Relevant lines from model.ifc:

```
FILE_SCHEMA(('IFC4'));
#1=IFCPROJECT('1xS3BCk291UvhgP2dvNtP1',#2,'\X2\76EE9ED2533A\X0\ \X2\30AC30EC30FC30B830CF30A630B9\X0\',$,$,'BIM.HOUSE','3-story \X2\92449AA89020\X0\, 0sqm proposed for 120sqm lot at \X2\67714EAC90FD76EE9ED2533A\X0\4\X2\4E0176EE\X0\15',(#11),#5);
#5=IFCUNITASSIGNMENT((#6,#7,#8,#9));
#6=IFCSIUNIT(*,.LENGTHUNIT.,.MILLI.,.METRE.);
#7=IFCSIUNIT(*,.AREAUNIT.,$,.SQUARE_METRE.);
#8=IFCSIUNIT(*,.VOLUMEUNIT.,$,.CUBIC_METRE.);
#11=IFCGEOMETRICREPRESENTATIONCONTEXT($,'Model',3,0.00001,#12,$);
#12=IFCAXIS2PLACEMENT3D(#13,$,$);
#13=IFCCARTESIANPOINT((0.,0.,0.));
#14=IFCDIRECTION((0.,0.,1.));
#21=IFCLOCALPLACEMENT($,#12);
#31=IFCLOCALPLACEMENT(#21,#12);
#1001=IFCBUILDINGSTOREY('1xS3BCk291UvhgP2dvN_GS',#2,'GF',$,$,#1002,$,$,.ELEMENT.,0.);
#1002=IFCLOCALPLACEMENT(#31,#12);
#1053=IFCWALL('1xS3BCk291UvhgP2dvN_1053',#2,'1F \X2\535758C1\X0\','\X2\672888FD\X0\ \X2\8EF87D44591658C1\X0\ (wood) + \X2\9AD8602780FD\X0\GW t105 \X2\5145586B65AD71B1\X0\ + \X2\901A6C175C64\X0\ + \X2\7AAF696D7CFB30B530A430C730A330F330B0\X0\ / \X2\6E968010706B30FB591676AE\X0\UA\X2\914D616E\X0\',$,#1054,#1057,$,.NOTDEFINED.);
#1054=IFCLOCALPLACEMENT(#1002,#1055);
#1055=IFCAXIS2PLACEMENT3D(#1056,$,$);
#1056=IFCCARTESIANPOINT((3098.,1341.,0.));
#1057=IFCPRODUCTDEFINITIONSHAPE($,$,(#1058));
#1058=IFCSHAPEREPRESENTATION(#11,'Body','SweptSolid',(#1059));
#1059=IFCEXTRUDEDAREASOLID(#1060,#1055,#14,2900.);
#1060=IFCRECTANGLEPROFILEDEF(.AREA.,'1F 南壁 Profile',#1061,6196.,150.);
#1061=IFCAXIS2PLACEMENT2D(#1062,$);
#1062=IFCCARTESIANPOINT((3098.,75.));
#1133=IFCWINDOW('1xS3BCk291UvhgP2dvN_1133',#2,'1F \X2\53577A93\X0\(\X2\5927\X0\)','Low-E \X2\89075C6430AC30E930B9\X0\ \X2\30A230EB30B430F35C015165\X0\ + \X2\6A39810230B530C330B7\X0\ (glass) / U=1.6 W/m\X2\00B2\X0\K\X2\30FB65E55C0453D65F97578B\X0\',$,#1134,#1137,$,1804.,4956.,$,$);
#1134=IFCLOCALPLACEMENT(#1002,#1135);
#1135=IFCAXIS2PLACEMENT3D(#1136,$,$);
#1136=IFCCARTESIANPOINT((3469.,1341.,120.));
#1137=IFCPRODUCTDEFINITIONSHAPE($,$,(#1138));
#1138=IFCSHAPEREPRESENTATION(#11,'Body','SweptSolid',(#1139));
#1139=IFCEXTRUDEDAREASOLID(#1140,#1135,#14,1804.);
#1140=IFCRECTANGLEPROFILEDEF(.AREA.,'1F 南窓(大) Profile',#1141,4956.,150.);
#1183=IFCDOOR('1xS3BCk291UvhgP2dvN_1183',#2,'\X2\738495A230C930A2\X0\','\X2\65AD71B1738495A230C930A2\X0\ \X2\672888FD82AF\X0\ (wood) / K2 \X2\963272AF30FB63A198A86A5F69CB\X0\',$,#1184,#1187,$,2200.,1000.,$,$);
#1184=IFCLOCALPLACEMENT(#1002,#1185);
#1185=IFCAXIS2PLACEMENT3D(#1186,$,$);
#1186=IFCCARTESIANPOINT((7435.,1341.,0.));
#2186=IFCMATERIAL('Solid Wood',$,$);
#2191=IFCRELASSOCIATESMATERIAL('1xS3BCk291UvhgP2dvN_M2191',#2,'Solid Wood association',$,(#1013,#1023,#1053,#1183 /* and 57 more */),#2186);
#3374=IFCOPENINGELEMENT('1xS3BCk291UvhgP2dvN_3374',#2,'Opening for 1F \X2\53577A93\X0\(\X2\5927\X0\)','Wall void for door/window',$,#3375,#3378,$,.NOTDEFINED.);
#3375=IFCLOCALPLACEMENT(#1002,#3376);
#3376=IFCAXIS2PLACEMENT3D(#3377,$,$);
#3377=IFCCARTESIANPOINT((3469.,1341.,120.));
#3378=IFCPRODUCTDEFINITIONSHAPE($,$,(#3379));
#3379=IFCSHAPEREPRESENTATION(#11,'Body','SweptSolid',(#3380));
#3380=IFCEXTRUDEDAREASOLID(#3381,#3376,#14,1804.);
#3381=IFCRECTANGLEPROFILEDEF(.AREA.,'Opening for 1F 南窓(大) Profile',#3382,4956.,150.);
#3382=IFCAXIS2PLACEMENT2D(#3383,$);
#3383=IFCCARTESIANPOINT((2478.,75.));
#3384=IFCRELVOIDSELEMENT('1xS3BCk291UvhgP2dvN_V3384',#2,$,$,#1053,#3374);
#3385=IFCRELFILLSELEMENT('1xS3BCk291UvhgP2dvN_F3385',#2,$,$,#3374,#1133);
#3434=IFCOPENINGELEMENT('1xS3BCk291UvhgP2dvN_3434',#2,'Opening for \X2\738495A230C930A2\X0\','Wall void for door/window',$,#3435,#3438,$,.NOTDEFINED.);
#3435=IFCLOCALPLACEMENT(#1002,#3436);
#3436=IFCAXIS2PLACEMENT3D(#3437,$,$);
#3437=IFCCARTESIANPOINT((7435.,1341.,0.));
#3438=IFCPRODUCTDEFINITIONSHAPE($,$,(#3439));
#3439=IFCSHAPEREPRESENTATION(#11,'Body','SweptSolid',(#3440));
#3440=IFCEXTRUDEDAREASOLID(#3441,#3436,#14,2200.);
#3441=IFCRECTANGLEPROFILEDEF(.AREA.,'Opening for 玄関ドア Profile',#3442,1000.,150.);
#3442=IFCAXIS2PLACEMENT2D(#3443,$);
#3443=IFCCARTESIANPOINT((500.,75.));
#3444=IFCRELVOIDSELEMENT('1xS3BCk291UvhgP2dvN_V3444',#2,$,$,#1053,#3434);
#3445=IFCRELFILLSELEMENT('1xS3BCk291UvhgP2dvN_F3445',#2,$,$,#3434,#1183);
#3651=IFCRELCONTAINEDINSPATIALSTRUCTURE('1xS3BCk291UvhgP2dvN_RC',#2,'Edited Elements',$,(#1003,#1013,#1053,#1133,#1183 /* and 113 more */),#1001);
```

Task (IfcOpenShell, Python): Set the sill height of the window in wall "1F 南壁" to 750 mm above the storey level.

```python
import numpy as np
import ifcopenshell
import ifcopenshell.api.geometry
import ifcopenshell.geom
import ifcopenshell.util.element
import ifcopenshell.util.placement
import ifcopenshell.util.shape
import ifcopenshell.util.unit

model = ifcopenshell.open("model.ifc")
unit_scale = ifcopenshell.util.unit.calculate_unit_scale(model)

window = model.by_id(1133)
opening = window.FillsVoids[0].RelatingOpeningElement
storey = ifcopenshell.util.element.get_container(window, ifc_class="IfcBuildingStorey")
level = ifcopenshell.util.placement.get_local_placement(storey.ObjectPlacement)[2, 3]

# The opening's origin need not be at the sill, so measure its lowest point.
shape = ifcopenshell.geom.create_shape(ifcopenshell.geom.settings(), opening)
bottom = ifcopenshell.util.shape.get_shape_bottom_elevation(shape, shape.geometry) / unit_scale
dz = level + 0.75 / unit_scale - bottom

shift = np.array([0.0, 0.0, dz])
# The window is not placed relative to its opening, so move both.
for product in (opening, window):
    matrix = ifcopenshell.util.placement.get_local_placement(product.ObjectPlacement)
    matrix[:3, 3] += shift
    ifcopenshell.api.geometry.edit_object_placement(model, product=product, matrix=matrix, is_si=False)

print(f"moved by {dz * unit_scale:+.3f} m")

model.write("model-out.ifc")
```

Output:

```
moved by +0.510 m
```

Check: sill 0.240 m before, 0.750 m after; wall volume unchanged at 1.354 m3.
